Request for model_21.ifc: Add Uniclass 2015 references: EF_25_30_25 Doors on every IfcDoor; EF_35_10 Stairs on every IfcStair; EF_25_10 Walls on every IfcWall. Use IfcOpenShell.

First a look at what the model holds.

```python
import ifcopenshell

model = ifcopenshell.open("model_21.ifc")
print(model.schema)
print("classifications:", [c.Name for c in model.by_type("IfcClassification")])
for ifc_class in ("IfcDoor", "IfcRoof", "IfcStair", "IfcWall", "IfcWindow"):
    print(ifc_class, len(model.by_type(ifc_class)))
```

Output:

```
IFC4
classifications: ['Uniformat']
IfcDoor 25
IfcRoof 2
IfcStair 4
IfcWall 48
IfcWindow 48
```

```python
import ifcopenshell
import ifcopenshell.api.classification

model = ifcopenshell.open("model_21.ifc")

system = ifcopenshell.api.classification.add_classification(model, classification="Uniclass 2015")

codes = {
    "IfcDoor": ("EF_25_30_25", "Doors"),
    "IfcStair": ("EF_35_10", "Stairs"),
    "IfcWall": ("EF_25_10", "Walls"),
}
for ifc_class, (code, name) in codes.items():
    products = model.by_type(ifc_class)
    ifcopenshell.api.classification.add_reference(
        model, products=products, classification=system, identification=code, name=name
    )
    print(code, len(products))

model.write("model_21-out.ifc")
```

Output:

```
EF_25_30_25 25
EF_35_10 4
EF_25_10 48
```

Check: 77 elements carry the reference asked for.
